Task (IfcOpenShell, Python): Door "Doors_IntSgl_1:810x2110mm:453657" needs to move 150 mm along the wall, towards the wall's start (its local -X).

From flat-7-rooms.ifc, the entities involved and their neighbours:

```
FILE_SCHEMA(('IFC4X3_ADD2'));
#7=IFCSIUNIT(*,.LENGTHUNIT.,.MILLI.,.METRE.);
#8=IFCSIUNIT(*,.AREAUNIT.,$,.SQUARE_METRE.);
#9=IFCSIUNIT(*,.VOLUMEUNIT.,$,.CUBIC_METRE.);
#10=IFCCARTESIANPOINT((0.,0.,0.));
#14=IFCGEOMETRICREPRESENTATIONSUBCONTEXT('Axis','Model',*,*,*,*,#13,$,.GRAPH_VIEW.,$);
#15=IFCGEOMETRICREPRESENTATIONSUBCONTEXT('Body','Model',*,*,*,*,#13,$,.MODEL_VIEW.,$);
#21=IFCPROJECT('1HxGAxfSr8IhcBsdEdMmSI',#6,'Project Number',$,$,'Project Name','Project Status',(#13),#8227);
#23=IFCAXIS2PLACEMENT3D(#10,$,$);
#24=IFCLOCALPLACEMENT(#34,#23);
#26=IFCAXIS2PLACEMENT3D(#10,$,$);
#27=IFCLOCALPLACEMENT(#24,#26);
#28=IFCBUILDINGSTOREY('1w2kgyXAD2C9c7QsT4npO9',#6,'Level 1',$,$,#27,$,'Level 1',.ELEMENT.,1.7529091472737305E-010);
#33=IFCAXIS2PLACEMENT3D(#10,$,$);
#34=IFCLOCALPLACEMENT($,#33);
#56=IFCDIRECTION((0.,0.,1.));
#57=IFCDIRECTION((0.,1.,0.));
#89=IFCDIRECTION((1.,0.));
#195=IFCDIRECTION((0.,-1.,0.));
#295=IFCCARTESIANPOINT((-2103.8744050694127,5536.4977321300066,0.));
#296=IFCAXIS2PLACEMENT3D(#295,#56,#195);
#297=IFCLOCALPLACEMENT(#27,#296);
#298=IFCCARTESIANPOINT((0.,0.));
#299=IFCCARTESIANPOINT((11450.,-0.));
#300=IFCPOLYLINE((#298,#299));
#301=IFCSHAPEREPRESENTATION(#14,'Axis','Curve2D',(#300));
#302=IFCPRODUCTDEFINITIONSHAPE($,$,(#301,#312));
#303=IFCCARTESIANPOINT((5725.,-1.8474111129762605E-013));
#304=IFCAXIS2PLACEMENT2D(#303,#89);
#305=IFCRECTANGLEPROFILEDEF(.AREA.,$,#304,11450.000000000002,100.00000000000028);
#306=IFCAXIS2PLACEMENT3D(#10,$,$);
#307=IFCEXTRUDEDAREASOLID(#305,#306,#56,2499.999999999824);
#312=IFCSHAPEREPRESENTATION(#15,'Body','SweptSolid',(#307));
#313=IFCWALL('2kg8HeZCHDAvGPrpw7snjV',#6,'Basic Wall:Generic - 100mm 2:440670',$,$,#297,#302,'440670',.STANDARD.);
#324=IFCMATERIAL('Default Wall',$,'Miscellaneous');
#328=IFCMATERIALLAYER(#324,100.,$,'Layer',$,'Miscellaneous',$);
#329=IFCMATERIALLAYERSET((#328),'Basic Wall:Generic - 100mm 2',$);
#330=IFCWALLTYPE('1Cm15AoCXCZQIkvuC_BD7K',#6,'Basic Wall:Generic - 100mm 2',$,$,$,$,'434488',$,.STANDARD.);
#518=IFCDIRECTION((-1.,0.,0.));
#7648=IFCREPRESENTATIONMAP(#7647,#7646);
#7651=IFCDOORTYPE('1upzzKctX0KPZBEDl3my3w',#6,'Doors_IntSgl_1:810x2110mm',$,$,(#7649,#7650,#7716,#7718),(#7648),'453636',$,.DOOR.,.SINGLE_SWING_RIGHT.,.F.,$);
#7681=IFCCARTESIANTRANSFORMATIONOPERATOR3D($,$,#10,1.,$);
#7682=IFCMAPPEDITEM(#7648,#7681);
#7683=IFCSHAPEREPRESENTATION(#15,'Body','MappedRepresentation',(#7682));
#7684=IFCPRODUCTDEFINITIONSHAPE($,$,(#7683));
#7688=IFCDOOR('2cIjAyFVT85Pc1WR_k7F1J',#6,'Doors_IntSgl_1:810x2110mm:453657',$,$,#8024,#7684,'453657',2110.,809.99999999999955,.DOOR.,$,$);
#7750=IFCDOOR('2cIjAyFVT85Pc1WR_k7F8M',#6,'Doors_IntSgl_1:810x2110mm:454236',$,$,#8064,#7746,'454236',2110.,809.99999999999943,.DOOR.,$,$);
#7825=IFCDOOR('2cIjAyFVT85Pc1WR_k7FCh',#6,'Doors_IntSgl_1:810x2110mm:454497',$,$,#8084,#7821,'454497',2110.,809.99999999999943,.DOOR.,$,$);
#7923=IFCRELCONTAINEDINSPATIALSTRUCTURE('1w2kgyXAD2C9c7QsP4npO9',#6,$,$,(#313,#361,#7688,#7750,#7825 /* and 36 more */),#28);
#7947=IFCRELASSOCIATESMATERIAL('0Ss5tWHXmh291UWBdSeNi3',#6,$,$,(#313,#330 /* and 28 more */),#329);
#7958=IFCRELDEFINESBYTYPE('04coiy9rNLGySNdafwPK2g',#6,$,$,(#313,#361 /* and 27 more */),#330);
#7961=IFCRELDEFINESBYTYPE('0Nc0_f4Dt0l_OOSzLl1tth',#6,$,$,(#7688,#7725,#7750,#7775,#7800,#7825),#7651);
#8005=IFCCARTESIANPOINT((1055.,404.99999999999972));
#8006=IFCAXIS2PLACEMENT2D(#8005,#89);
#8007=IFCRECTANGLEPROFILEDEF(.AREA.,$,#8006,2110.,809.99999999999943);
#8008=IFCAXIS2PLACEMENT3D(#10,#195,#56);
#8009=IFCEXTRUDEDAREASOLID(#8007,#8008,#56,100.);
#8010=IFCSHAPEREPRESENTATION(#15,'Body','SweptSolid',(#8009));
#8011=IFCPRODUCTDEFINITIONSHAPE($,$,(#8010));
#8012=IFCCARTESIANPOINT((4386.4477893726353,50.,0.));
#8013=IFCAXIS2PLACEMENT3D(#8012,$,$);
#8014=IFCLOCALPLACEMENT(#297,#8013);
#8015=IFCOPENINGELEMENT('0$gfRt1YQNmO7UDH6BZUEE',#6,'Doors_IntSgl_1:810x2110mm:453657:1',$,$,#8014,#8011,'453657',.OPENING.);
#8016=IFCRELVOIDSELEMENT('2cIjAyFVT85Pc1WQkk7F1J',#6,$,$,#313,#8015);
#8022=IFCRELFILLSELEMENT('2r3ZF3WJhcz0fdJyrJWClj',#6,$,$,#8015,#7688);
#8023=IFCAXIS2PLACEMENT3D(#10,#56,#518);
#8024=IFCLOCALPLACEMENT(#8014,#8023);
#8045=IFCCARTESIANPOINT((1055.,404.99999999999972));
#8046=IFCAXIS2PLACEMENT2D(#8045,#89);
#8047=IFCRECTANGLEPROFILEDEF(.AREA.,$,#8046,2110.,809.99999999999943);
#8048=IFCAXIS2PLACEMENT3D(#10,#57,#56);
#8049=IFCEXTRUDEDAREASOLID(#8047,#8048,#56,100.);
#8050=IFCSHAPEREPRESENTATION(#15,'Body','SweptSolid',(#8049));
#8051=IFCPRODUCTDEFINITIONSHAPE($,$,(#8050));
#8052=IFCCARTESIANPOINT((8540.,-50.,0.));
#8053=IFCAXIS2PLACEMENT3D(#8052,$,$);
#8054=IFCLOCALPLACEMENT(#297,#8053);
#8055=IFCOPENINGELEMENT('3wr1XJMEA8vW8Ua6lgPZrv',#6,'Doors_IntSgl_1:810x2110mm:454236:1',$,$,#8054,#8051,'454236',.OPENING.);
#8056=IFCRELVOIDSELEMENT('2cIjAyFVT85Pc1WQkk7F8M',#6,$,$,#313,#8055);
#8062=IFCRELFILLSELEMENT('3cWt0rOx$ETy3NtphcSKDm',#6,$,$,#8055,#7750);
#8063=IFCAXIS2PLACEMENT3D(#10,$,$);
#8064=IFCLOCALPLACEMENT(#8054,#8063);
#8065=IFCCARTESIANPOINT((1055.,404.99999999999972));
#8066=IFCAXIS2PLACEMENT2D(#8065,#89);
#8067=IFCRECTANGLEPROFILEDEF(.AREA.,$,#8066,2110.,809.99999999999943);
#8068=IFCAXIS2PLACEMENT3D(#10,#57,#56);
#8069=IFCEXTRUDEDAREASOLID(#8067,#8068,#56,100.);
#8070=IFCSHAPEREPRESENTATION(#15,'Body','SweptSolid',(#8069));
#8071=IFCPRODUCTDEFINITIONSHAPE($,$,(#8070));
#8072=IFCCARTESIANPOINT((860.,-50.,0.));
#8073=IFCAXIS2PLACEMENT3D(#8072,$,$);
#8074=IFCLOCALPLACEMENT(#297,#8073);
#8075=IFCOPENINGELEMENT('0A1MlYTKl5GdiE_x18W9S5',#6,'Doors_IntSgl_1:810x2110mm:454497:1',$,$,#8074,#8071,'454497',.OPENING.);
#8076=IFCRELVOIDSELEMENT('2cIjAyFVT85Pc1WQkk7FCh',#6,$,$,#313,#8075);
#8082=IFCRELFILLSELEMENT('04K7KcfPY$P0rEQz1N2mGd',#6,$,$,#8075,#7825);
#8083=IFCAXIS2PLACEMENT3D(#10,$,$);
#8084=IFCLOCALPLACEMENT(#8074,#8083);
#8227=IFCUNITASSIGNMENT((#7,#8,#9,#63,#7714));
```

```python
import ifcopenshell
import ifcopenshell.api.geometry
import ifcopenshell.util.placement

model = ifcopenshell.open("flat-7-rooms.ifc")

door = model.by_id(7688)
opening = door.FillsVoids[0].RelatingOpeningElement
wall = opening.VoidsElements[0].RelatingBuildingElement

wall_matrix = ifcopenshell.util.placement.get_local_placement(wall.ObjectPlacement)
shift = wall_matrix[:3, 0] * -150.0
before = ifcopenshell.util.placement.get_local_placement(door.ObjectPlacement)[:3, 3].copy()

# The door is placed relative to its opening, so it follows when the opening moves.
matrix = ifcopenshell.util.placement.get_local_placement(opening.ObjectPlacement)
matrix[:3, 3] += shift
ifcopenshell.api.geometry.edit_object_placement(
    model, product=opening, matrix=matrix, is_si=False, should_transform_children=True
)

after = ifcopenshell.util.placement.get_local_placement(door.ObjectPlacement)[:3, 3]
print("door moved by", (after - before).round(3) + 0.0)

model.write("flat-7-rooms_rev.ifc")
```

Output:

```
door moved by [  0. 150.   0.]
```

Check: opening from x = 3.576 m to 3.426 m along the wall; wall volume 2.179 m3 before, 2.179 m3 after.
